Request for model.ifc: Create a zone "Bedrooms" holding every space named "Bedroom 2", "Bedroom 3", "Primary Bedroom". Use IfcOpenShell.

First a look at what the model holds.

```python
import ifcopenshell

model = ifcopenshell.open("model.ifc")
print(model.schema)
seen = {}
for space in model.by_type("IfcSpace"):
    seen[space.LongName] = seen.get(space.LongName, 0) + 1
for name, count in sorted(seen.items(), key=str):
    print(count, "x", name)
print("zones:", [z.Name for z in model.by_type("IfcZone")][:20])
```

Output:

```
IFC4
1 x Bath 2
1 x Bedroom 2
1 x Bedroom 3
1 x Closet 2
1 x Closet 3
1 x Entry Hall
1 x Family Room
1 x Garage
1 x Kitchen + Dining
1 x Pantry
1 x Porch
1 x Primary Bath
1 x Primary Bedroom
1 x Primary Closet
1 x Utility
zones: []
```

```python
import ifcopenshell
import ifcopenshell.api.group
import ifcopenshell.api.root

model = ifcopenshell.open("model.ifc")

names = {"Bedroom 2", "Bedroom 3", "Primary Bedroom"}
spaces = [s for s in model.by_type("IfcSpace") if s.LongName in names]

zone = ifcopenshell.api.root.create_entity(model, ifc_class="IfcZone", name="Bedrooms")
ifcopenshell.api.group.assign_group(model, products=spaces, group=zone)
print(len(spaces), "spaces in", zone.Name)

model.write("model_rev.ifc")
```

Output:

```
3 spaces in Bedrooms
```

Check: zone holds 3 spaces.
